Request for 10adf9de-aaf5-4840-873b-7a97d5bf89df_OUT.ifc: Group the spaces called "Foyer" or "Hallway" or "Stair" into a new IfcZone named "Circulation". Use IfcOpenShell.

First a look at what the model holds.

```python
import ifcopenshell

model = ifcopenshell.open("10adf9de-aaf5-4840-873b-7a97d5bf89df_OUT.ifc")
print(model.schema)
seen = {}
for space in model.by_type("IfcSpace"):
    seen[space.LongName] = seen.get(space.LongName, 0) + 1
for name, count in sorted(seen.items(), key=str):
    print(count, "x", name)
print("zones:", [z.Name for z in model.by_type("IfcZone")][:20])
```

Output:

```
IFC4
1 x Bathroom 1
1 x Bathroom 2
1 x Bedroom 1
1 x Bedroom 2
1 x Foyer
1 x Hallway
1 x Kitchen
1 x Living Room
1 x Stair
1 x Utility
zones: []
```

```python
import ifcopenshell
import ifcopenshell.api.group
import ifcopenshell.api.root

model = ifcopenshell.open("10adf9de-aaf5-4840-873b-7a97d5bf89df_OUT.ifc")

names = {"Foyer", "Hallway", "Stair"}
spaces = [s for s in model.by_type("IfcSpace") if s.LongName in names]

zone = ifcopenshell.api.root.create_entity(model, ifc_class="IfcZone", name="Circulation")
ifcopenshell.api.group.assign_group(model, products=spaces, group=zone)
print(len(spaces), "spaces in", zone.Name)

model.write("10adf9de-aaf5-4840-873b-7a97d5bf89df_OUT_updated.ifc")
```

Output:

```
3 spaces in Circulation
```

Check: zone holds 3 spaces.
